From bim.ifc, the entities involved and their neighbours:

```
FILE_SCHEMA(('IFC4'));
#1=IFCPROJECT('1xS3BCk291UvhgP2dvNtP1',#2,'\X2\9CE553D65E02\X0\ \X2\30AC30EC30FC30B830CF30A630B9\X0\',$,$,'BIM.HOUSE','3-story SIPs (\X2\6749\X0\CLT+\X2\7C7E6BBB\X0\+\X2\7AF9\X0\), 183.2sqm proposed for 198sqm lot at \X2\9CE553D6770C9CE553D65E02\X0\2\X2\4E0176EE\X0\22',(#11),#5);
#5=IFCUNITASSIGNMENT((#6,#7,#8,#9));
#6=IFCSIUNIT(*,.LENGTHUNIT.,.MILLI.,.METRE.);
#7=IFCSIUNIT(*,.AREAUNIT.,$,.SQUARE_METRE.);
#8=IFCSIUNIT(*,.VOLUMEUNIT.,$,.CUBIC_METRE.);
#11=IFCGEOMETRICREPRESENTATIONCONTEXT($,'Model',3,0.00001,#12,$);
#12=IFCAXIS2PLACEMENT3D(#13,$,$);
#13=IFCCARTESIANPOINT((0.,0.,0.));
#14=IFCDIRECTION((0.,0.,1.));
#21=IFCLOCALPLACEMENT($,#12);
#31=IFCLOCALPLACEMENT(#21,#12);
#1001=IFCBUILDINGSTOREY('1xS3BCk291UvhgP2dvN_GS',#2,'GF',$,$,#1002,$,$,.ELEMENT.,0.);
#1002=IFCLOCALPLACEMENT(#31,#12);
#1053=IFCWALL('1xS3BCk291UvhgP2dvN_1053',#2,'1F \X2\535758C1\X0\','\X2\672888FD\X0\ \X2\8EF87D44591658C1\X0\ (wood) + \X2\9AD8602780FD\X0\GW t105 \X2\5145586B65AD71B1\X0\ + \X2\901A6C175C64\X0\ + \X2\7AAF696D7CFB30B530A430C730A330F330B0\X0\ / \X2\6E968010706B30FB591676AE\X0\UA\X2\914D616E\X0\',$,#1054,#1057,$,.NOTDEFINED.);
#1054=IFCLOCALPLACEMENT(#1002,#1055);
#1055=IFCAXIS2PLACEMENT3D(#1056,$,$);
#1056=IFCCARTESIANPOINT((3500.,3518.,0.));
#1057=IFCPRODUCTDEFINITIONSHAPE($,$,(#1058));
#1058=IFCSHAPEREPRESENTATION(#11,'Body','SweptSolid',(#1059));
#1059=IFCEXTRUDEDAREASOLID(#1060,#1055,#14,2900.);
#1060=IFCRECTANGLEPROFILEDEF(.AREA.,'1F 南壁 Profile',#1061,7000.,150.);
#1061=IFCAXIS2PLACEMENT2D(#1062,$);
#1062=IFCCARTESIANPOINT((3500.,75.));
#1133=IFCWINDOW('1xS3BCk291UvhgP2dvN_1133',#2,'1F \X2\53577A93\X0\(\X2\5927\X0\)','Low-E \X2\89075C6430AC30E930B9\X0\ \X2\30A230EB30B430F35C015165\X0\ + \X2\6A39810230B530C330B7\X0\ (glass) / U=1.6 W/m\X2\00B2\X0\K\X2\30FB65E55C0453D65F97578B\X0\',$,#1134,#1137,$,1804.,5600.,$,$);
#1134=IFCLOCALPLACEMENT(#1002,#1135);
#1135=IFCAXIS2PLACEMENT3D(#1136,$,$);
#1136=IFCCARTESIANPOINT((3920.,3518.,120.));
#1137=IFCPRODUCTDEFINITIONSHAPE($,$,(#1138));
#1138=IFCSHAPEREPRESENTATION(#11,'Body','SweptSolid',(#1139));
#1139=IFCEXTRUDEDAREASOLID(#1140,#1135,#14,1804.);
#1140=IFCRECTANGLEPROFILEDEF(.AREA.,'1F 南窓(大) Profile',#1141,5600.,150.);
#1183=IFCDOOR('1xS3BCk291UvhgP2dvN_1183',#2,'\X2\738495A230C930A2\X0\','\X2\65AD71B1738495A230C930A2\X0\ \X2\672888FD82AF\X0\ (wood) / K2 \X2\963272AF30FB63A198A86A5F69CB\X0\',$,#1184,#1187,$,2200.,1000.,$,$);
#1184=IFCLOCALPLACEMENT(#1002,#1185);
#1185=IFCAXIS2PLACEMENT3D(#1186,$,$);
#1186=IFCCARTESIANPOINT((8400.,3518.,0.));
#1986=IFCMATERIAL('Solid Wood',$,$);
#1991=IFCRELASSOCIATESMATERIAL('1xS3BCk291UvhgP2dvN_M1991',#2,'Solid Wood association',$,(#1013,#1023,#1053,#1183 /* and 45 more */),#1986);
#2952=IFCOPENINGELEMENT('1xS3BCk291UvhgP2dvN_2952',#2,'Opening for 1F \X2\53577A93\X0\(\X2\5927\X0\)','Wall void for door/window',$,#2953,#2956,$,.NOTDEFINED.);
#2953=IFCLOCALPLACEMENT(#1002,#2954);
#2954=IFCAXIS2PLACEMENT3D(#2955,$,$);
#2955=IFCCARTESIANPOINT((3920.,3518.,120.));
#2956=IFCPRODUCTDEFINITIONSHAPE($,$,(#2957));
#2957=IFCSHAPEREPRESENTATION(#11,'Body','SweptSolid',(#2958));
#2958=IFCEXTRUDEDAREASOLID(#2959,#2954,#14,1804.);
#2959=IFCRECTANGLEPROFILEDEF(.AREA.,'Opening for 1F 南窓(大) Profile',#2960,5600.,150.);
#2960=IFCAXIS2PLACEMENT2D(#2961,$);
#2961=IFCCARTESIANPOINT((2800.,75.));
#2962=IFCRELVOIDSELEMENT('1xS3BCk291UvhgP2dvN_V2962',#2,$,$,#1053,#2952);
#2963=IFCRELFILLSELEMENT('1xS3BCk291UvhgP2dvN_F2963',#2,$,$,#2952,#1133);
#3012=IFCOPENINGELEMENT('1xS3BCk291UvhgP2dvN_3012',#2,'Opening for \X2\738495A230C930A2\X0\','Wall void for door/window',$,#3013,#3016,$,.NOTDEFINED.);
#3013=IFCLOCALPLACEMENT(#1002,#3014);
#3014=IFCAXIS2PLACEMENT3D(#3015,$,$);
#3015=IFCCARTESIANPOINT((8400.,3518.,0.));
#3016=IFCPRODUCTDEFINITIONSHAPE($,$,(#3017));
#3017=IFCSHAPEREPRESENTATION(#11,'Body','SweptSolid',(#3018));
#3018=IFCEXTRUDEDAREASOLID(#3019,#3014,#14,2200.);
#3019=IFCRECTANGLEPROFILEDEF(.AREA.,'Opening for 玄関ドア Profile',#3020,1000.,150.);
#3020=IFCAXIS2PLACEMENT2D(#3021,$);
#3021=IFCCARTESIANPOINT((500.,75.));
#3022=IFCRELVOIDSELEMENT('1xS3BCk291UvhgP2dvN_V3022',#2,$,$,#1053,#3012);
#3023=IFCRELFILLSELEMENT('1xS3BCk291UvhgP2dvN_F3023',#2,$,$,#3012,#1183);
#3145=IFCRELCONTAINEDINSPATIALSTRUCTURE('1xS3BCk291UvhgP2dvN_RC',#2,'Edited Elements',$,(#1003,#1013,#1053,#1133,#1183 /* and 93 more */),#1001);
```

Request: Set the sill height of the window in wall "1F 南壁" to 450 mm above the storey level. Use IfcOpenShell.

```python
import numpy as np
import ifcopenshell
import ifcopenshell.api.geometry
import ifcopenshell.geom
import ifcopenshell.util.element
import ifcopenshell.util.placement
import ifcopenshell.util.shape
import ifcopenshell.util.unit

model = ifcopenshell.open("bim.ifc")
unit_scale = ifcopenshell.util.unit.calculate_unit_scale(model)

window = model.by_guid("1xS3BCk291UvhgP2dvN_1133")
opening = window.FillsVoids[0].RelatingOpeningElement
storey = ifcopenshell.util.element.get_container(window, ifc_class="IfcBuildingStorey")
level = ifcopenshell.util.placement.get_local_placement(storey.ObjectPlacement)[2, 3]

# The opening's origin need not be at the sill, so measure its lowest point.
shape = ifcopenshell.geom.create_shape(ifcopenshell.geom.settings(), opening)
bottom = ifcopenshell.util.shape.get_shape_bottom_elevation(shape, shape.geometry) / unit_scale
dz = level + 0.45 / unit_scale - bottom

shift = np.array([0.0, 0.0, dz])
# The window is not placed relative to its opening, so move both.
for product in (opening, window):
    matrix = ifcopenshell.util.placement.get_local_placement(product.ObjectPlacement)
    matrix[:3, 3] += shift
    ifcopenshell.api.geometry.edit_object_placement(model, product=product, matrix=matrix, is_si=False)

print(f"moved by {dz * unit_scale:+.3f} m")

model.write("bim_v2.ifc")
```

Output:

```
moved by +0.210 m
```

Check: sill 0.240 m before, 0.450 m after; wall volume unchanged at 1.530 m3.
